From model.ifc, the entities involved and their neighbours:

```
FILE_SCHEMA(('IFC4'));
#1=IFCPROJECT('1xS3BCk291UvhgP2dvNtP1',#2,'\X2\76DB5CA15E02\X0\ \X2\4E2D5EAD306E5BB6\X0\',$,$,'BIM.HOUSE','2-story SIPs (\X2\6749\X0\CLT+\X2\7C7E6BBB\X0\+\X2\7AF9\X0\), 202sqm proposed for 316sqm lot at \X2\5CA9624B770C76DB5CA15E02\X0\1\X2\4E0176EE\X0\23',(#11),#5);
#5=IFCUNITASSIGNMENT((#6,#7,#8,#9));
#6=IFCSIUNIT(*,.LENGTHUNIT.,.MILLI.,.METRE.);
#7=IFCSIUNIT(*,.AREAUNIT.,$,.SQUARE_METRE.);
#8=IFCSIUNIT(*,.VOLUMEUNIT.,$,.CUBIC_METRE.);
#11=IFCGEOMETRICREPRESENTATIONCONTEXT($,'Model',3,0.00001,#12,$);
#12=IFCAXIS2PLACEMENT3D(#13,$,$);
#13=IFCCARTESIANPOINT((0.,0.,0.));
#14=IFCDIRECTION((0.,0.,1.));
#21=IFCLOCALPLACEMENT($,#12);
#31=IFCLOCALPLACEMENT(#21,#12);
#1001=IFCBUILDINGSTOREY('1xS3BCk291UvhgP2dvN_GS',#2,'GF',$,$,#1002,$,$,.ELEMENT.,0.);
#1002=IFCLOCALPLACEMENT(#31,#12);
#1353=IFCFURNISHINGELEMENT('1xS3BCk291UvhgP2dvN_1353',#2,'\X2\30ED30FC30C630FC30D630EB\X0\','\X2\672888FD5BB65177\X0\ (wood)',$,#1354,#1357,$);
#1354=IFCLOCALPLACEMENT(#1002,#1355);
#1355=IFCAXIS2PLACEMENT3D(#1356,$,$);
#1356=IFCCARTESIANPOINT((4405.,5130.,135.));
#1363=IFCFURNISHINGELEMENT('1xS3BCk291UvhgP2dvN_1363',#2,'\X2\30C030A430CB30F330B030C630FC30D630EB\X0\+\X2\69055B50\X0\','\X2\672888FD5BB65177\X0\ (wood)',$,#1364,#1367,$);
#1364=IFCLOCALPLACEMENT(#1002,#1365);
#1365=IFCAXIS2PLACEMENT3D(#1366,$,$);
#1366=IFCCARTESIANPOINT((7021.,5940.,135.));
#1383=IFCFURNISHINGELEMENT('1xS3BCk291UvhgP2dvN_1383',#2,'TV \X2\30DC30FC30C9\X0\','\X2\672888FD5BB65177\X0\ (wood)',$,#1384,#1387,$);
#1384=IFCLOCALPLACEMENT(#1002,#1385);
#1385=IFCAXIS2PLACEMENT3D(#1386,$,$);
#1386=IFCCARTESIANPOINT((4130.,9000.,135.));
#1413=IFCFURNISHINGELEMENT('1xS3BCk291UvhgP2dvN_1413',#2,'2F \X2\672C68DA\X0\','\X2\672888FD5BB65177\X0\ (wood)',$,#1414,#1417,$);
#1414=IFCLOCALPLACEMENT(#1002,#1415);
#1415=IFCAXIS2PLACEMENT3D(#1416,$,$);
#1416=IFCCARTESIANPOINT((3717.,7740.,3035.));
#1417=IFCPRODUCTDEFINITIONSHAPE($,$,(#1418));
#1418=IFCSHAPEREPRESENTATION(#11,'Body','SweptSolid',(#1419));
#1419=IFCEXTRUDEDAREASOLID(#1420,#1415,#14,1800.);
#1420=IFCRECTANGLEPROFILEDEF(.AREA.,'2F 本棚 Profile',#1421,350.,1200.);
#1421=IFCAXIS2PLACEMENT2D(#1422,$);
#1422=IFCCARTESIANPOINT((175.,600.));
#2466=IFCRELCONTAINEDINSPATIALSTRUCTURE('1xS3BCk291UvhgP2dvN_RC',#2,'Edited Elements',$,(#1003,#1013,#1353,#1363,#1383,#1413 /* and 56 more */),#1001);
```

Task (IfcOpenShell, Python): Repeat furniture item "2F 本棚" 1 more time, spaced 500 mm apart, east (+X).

```python
import numpy as np
import ifcopenshell
import ifcopenshell.api.geometry
import ifcopenshell.api.root
import ifcopenshell.util.element
import ifcopenshell.util.placement

model = ifcopenshell.open("model.ifc")


def reuse_history(source, copy):
    """copy_class also copies each property set's owner history, people and application; keep the originals."""
    for rel in copy.IsDefinedBy:
        if rel.is_a("IfcRelDefinesByProperties") and (history := rel.RelatingPropertyDefinition.OwnerHistory):
            rel.RelatingPropertyDefinition.OwnerHistory = source.OwnerHistory
            ifcopenshell.util.element.remove_deep2(model, history)


source = model.by_guid("1xS3BCk291UvhgP2dvN_1413")
base = ifcopenshell.util.placement.get_local_placement(source.ObjectPlacement)
step = np.array([1.0, 0.0, 0.0]) * 500.0

for i in range(1, 2):
    copy = ifcopenshell.api.root.copy_class(model, product=source)
    copy.Representation = ifcopenshell.util.element.copy_deep(
        model, source.Representation, exclude=["IfcGeometricRepresentationContext", "IfcRepresentationMap"]
    )
    reuse_history(source, copy)
    matrix = base.copy()
    matrix[:3, 3] += i * step
    print("added at", matrix[:3, 3].round(3) + 0.0)
    ifcopenshell.api.geometry.edit_object_placement(model, product=copy, matrix=matrix, is_si=False)

model.write("model_updated.ifc")
```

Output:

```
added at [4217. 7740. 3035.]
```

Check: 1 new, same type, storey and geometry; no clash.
